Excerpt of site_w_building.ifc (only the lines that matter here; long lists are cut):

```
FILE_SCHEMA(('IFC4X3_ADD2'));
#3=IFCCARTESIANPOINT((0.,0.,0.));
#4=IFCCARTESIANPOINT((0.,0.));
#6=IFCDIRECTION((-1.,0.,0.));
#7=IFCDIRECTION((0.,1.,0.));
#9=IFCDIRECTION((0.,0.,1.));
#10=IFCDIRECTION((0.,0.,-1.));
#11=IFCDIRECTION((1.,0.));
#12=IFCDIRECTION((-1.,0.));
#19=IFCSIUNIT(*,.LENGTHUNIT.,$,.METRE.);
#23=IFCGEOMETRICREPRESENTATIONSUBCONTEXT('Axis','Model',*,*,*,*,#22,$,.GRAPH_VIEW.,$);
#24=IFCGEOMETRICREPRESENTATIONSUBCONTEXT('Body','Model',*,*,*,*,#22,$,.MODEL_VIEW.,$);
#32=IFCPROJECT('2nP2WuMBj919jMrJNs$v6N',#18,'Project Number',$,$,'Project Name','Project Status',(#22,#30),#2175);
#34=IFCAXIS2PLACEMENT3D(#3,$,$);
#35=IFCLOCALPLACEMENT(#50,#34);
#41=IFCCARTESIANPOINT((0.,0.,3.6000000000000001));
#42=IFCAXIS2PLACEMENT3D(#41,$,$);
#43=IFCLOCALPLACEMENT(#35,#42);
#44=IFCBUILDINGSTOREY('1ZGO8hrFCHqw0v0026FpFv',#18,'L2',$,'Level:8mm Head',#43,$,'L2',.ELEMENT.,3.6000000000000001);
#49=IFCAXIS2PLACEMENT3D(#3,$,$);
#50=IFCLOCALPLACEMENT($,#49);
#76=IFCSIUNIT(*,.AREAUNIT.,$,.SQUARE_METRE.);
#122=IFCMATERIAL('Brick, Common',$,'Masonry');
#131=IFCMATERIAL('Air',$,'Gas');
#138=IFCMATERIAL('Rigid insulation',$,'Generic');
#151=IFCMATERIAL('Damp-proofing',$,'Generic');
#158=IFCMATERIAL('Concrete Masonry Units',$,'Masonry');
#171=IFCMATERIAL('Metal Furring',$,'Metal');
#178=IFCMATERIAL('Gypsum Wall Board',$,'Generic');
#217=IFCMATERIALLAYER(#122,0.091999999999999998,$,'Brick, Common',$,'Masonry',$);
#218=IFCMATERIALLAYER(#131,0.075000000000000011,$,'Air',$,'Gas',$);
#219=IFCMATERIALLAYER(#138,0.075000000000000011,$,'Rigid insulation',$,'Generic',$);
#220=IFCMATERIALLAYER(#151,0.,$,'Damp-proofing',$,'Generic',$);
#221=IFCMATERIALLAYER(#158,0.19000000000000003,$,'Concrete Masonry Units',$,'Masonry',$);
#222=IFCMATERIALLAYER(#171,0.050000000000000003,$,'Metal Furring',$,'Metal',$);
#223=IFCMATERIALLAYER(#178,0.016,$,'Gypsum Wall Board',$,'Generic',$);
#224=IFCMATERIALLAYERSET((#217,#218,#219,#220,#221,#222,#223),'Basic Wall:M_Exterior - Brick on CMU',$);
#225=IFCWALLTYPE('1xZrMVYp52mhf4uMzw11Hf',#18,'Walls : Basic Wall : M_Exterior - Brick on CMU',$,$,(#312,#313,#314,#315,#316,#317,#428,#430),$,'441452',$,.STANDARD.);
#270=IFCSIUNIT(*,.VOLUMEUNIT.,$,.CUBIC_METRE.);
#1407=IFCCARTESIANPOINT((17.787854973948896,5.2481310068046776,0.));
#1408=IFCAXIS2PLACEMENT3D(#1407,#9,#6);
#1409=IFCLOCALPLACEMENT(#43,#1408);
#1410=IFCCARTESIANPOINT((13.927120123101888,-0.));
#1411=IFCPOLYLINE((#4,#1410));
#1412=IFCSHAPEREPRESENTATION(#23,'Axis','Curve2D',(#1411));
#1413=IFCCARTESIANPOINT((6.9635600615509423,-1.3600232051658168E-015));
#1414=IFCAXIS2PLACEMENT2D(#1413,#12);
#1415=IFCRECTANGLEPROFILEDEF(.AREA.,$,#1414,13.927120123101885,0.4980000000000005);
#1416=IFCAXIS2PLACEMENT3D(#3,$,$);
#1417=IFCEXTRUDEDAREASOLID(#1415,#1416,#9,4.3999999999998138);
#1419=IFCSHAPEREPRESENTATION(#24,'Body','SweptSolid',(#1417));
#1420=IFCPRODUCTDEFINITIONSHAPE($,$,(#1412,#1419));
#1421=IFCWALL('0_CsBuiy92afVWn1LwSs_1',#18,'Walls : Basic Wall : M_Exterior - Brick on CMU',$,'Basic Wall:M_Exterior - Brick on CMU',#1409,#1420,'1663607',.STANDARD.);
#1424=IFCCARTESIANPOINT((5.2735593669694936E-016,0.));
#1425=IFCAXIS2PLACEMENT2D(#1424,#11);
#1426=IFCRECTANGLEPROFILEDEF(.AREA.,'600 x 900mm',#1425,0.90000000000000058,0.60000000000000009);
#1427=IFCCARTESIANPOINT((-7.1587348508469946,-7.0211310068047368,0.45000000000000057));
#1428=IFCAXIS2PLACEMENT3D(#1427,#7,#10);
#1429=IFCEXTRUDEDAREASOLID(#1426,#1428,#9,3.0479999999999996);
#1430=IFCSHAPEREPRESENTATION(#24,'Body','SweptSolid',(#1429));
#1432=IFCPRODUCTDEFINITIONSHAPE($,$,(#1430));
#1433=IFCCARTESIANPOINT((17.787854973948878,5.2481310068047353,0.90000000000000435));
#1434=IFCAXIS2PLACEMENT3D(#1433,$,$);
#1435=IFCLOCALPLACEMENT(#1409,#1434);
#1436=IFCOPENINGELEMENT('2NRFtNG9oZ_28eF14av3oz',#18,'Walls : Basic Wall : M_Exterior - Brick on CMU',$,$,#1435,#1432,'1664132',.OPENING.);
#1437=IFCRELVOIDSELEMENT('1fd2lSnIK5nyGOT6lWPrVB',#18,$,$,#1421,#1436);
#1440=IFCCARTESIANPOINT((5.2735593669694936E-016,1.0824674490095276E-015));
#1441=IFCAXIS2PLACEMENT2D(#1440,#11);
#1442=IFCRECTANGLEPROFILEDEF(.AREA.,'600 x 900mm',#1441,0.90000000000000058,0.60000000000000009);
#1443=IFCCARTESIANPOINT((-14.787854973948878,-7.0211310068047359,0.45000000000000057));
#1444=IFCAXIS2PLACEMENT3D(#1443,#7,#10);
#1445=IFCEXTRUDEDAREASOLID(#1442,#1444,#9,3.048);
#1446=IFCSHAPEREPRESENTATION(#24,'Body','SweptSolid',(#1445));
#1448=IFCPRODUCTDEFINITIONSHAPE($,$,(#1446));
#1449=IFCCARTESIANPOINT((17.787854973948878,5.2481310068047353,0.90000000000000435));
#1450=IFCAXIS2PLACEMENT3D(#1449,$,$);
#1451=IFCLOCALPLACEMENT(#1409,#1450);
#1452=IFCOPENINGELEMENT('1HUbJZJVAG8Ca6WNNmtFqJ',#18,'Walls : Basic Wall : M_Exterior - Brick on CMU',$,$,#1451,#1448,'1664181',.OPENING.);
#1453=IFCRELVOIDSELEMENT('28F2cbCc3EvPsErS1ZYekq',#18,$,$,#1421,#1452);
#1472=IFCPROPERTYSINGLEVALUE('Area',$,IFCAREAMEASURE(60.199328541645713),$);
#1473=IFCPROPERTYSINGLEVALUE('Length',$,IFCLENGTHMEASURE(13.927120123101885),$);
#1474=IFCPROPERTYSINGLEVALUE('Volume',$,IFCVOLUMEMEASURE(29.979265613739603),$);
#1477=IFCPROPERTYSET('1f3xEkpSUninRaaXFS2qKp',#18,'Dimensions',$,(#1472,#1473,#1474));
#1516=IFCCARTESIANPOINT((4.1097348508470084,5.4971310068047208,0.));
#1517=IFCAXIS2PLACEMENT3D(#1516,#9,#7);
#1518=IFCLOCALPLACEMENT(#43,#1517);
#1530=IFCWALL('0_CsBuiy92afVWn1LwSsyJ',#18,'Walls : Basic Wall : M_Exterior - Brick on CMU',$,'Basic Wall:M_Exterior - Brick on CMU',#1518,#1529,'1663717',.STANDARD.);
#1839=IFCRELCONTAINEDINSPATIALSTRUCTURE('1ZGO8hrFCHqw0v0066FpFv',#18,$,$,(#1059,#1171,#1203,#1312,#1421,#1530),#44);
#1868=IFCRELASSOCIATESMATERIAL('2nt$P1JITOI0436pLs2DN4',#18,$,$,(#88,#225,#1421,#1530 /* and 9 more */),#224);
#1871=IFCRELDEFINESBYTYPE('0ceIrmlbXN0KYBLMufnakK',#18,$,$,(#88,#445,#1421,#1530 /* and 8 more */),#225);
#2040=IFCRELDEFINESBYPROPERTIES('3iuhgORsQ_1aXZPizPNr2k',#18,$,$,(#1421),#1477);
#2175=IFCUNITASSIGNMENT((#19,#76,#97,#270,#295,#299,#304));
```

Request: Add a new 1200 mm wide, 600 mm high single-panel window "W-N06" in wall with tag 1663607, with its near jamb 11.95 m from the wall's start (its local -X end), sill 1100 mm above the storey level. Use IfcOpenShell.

```python
import numpy as np
import ifcopenshell
import ifcopenshell.api.feature
import ifcopenshell.api.geometry
import ifcopenshell.api.pset
import ifcopenshell.api.root
import ifcopenshell.api.spatial
import ifcopenshell.geom
import ifcopenshell.util.element
import ifcopenshell.util.placement
import ifcopenshell.util.representation
import ifcopenshell.util.shape
import ifcopenshell.util.unit

model = ifcopenshell.open("site_w_building.ifc")
unit_scale = ifcopenshell.util.unit.calculate_unit_scale(model)
area_scale = ifcopenshell.util.unit.calculate_unit_scale(model, "AREAUNIT")
volume_scale = ifcopenshell.util.unit.calculate_unit_scale(model, "VOLUMEUNIT")
settings = ifcopenshell.geom.settings()


def volume(element):
    """Net volume in cubic metres, openings subtracted."""
    shape = ifcopenshell.geom.create_shape(settings, element)
    return ifcopenshell.util.shape.get_volume(shape.geometry)


wall = model.by_id(1421)
storey = ifcopenshell.util.element.get_container(wall, ifc_class="IfcBuildingStorey")
context = ifcopenshell.util.representation.get_context(model, "Model", "Body", "MODEL_VIEW")
before = volume(wall)

width, height, from_end, sill = 1.2, 0.6, 11.95, 1.1  # metres

# The wall runs along its own X axis, and the end named is its -X end.
wall_shape = ifcopenshell.geom.create_shape(settings, wall)
x, y, z = ifcopenshell.util.shape.get_vertices(wall_shape.geometry).T
start = x.min() + from_end
face, thickness = float(y.min()), float(y.max() - y.min())
wall_matrix = ifcopenshell.util.placement.get_local_placement(wall.ObjectPlacement)
level = ifcopenshell.util.placement.get_local_placement(storey.ObjectPlacement)[2, 3]


def in_wall(x, y):
    """Placement at x, y metres in the wall's axes, at sill height."""
    matrix = wall_matrix.copy()
    matrix[:, 3] = wall_matrix @ np.array([x / unit_scale, y / unit_scale, 0.0, 1.0])
    matrix[2, 3] = level + sill / unit_scale
    return matrix


# Opening: a box that overshoots both wall faces by 50 mm.
opening = ifcopenshell.api.root.create_entity(model, ifc_class="IfcOpeningElement", predefined_type="OPENING")
box = ifcopenshell.api.geometry.add_wall_representation(
    model, context=context, length=width, height=height, thickness=thickness + 0.1
)
ifcopenshell.api.geometry.assign_representation(model, product=opening, representation=box)
ifcopenshell.api.geometry.edit_object_placement(model, product=opening, matrix=in_wall(start, face - 0.05), is_si=False)
ifcopenshell.api.feature.add_feature(model, feature=opening, element=wall)

window = ifcopenshell.api.root.create_entity(model, ifc_class="IfcWindow", name="W-N06", predefined_type="WINDOW")
window.OverallWidth, window.OverallHeight = width / unit_scale, height / unit_scale
window.PartitioningType = "SINGLE_PANEL"
body = ifcopenshell.api.geometry.add_window_representation(
    model,
    context=context,
    overall_width=window.OverallWidth,
    overall_height=window.OverallHeight,
    partition_type="SINGLE_PANEL",
)
ifcopenshell.api.geometry.assign_representation(model, product=window, representation=body)
ifcopenshell.api.spatial.assign_container(model, products=[window], relating_structure=storey)
ifcopenshell.api.feature.add_filling(model, opening=opening, element=window)

# Centre the window in the wall's thickness.
ifcopenshell.api.geometry.edit_object_placement(model, product=window, matrix=in_wall(start, face), is_si=False)
window_shape = ifcopenshell.geom.create_shape(settings, window)
depth = ifcopenshell.util.shape.get_vertices(window_shape.geometry)[:, 1]
offset = face + thickness / 2 - (depth.min() + depth.max()) / 2
ifcopenshell.api.geometry.edit_object_placement(model, product=window, matrix=in_wall(start, offset), is_si=False)

after = volume(wall)

# Update the wall's stored quantities.
pset = model.by_id(ifcopenshell.util.element.get_pset(wall, "Dimensions", should_inherit=False)["id"])
ifcopenshell.api.pset.edit_pset(model, pset=pset, properties={
    "Area": model.create_entity("IfcAreaMeasure", after / thickness / area_scale),
    "Volume": model.create_entity("IfcVolumeMeasure", after / volume_scale),
})

print(f"wall volume {before:.3f} -> {after:.3f} m3")

model.write("site_w_building_rev.ifc")
```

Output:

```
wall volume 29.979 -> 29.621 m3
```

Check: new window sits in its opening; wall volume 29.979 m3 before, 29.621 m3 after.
